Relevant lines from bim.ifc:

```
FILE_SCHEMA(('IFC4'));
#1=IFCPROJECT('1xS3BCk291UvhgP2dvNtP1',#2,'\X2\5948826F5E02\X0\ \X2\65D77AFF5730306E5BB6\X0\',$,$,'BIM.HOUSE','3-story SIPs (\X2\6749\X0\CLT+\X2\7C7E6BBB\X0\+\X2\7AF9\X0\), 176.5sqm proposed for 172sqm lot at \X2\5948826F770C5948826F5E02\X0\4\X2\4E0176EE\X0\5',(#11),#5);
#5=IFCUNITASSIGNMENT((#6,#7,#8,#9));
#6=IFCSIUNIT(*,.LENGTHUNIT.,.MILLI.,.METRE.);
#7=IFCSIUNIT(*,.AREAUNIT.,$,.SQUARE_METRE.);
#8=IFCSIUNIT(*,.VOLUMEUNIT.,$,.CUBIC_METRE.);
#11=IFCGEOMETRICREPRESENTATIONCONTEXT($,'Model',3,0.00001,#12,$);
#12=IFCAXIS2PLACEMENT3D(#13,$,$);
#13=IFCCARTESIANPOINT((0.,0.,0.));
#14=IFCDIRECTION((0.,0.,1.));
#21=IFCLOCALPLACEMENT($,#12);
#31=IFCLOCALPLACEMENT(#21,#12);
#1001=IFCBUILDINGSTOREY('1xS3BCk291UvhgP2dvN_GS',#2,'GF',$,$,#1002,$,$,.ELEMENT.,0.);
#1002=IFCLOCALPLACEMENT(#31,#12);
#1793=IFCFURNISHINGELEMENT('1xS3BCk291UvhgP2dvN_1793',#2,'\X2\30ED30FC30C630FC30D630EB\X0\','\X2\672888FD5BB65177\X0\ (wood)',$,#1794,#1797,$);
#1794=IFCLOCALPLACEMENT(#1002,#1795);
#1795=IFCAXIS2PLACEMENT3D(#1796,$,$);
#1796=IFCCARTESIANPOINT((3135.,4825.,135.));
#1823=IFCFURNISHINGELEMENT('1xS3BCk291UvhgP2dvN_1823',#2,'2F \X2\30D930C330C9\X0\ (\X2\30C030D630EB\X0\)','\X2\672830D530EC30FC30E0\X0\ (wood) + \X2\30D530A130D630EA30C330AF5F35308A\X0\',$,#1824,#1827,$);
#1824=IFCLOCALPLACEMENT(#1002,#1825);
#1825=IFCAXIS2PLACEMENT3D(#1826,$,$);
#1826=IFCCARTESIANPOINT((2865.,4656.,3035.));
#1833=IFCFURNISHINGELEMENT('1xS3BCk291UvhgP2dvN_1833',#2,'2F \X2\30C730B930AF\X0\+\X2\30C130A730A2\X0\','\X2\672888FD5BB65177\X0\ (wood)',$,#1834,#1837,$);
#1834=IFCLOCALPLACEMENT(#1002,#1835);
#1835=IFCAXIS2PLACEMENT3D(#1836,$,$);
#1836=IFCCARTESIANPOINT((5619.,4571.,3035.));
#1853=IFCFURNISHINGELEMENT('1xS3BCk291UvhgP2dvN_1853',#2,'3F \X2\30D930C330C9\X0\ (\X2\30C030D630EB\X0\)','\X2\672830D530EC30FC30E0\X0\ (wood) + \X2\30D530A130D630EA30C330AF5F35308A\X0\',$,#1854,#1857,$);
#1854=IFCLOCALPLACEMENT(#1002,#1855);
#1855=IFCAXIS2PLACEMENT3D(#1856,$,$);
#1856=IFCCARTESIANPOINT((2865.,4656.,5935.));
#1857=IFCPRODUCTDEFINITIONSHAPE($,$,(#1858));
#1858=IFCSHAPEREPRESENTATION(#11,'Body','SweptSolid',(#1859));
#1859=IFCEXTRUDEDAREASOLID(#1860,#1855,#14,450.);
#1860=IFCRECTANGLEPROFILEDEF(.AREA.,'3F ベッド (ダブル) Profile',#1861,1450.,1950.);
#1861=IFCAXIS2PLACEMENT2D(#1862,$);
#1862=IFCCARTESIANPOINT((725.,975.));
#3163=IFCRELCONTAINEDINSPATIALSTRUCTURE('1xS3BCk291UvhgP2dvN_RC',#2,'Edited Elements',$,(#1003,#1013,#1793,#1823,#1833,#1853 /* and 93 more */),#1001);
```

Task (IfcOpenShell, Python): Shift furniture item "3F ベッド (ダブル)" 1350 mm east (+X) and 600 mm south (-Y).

```python
import ifcopenshell
import ifcopenshell.api.geometry
import ifcopenshell.util.placement
import ifcopenshell.util.unit

model = ifcopenshell.open("bim.ifc")
unit_scale = ifcopenshell.util.unit.calculate_unit_scale(model)

item = model.by_guid("1xS3BCk291UvhgP2dvN_1853")
matrix = ifcopenshell.util.placement.get_local_placement(item.ObjectPlacement)
matrix[0, 3] += 1.35 / unit_scale
matrix[1, 3] -= 0.6 / unit_scale
ifcopenshell.api.geometry.edit_object_placement(model, product=item, matrix=matrix, is_si=False)

print(ifcopenshell.util.placement.get_local_placement(item.ObjectPlacement).round(3) + 0.0)

model.write("bim_v2.ifc")
```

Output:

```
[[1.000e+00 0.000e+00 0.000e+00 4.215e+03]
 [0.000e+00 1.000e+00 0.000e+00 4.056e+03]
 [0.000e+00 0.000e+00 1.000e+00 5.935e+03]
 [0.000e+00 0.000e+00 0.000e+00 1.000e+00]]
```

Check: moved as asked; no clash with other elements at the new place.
